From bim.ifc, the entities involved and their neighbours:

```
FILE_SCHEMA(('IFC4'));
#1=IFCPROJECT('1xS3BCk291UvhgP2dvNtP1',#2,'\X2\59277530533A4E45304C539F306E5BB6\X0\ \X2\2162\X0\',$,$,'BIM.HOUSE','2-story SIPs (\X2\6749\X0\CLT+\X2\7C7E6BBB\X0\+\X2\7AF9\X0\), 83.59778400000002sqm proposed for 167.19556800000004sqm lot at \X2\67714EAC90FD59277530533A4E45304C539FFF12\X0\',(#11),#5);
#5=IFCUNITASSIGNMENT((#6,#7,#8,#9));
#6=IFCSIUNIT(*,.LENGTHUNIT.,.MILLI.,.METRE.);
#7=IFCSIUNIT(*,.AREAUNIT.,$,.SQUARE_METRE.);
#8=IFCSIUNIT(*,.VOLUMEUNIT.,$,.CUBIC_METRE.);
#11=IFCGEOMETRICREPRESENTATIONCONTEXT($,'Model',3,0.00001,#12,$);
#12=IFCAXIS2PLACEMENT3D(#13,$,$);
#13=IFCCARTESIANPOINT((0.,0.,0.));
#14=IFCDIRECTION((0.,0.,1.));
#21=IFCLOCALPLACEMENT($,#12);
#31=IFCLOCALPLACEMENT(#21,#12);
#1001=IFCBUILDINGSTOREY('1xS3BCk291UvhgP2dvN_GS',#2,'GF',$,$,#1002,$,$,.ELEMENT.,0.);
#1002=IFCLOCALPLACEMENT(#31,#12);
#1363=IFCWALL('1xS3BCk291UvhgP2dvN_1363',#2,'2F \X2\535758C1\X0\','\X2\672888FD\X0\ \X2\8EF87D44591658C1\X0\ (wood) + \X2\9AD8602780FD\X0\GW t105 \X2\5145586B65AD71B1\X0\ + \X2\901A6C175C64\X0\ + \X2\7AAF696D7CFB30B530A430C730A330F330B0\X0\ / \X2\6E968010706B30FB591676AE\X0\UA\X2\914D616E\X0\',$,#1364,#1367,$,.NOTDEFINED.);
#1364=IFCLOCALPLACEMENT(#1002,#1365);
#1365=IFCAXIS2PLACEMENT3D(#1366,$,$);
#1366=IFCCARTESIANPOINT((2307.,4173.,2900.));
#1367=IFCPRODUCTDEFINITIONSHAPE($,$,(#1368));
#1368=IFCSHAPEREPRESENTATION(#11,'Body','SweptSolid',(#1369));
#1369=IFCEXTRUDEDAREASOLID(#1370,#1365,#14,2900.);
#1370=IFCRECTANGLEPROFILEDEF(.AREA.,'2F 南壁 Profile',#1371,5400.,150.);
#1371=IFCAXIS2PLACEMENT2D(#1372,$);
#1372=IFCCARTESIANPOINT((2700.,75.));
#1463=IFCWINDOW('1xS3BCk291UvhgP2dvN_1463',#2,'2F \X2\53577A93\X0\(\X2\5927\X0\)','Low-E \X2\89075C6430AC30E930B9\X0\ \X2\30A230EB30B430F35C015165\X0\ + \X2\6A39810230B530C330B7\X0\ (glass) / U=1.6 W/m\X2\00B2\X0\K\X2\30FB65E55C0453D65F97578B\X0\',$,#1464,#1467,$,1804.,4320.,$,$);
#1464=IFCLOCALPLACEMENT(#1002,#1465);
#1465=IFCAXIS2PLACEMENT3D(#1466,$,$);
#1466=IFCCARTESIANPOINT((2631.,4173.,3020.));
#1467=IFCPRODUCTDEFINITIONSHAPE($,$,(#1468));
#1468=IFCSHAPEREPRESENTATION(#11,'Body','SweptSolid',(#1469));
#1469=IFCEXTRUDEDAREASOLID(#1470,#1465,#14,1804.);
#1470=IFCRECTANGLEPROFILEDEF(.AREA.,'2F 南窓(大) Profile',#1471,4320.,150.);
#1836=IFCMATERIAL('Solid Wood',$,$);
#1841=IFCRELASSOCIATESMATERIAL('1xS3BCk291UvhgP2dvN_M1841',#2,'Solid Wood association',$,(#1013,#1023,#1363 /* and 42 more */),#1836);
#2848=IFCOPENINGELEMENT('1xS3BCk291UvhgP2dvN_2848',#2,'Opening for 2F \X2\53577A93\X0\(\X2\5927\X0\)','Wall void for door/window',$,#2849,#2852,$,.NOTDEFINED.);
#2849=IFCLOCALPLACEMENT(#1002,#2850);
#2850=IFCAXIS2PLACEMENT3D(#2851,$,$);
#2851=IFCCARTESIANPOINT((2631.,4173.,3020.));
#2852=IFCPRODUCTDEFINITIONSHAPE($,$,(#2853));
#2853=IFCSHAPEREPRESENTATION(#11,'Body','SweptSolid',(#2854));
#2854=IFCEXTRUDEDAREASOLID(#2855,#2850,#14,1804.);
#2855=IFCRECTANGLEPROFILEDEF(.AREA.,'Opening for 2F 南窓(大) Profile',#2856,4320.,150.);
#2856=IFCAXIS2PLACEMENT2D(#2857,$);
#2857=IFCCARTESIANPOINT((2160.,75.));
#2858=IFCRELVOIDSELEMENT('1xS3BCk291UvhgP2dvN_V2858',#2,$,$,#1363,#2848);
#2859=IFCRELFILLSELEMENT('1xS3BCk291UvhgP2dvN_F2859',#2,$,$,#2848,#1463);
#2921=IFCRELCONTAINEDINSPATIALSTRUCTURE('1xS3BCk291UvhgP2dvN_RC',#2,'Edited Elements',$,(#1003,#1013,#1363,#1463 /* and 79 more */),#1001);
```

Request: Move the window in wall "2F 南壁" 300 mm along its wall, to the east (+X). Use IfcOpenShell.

```python
import ifcopenshell
import ifcopenshell.api.geometry
import ifcopenshell.util.placement

model = ifcopenshell.open("bim.ifc")

window = model.by_guid("1xS3BCk291UvhgP2dvN_1463")
opening = window.FillsVoids[0].RelatingOpeningElement
wall = opening.VoidsElements[0].RelatingBuildingElement

wall_matrix = ifcopenshell.util.placement.get_local_placement(wall.ObjectPlacement)
shift = wall_matrix[:3, 0] * 300.0
before = ifcopenshell.util.placement.get_local_placement(window.ObjectPlacement)[:3, 3].copy()

# The window is not placed relative to its opening, so move both.
for product in (opening, window):
    matrix = ifcopenshell.util.placement.get_local_placement(product.ObjectPlacement)
    matrix[:3, 3] += shift
    ifcopenshell.api.geometry.edit_object_placement(model, product=product, matrix=matrix, is_si=False)

after = ifcopenshell.util.placement.get_local_placement(window.ObjectPlacement)[:3, 3]
print("window moved by", (after - before).round(3) + 0.0)

model.write("bim_rev.ifc")
```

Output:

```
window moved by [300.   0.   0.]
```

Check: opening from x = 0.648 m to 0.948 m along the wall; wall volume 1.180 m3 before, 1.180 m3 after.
